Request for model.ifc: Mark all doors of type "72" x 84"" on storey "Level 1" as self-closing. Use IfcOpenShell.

First a look at what the model holds.

```python
import ifcopenshell
import ifcopenshell.util.element

model = ifcopenshell.open("model.ifc")
print(model.schema)
storey = next(s for s in model.by_type("IfcBuildingStorey") if s.Name == "Level 1")
doors = [e for e in ifcopenshell.util.element.get_decomposition(storey) if e.is_a("IfcDoor")]
seen = {}
for e in doors:
    element_type = ifcopenshell.util.element.get_type(e)
    key = (element_type.Name if element_type != e and element_type else None, ifcopenshell.util.element.get_pset(e, "Pset_DoorCommon", "SelfClosing"))
    seen[key] = seen.get(key, 0) + 1
for (name, value), count in sorted(seen.items(), key=str):
    print(count, "x", name, "|", value)
```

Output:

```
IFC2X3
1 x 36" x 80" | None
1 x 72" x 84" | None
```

```python
import ifcopenshell
import ifcopenshell.api.pset
import ifcopenshell.util.element

model = ifcopenshell.open("model.ifc")

storey = next(s for s in model.by_type("IfcBuildingStorey") if s.Name == "Level 1")
doors = [e for e in ifcopenshell.util.element.get_decomposition(storey) if e.is_a("IfcDoor")]

count = 0
for e in doors:
    element_type = ifcopenshell.util.element.get_type(e)
    if element_type in (None, e) or element_type.Name != '72" x 84"':
        continue
    # add_pset returns the element's existing set when there is one.
    pset = ifcopenshell.api.pset.add_pset(model, product=e, name="Pset_DoorCommon")
    ifcopenshell.api.pset.edit_pset(model, pset=pset, properties={"SelfClosing": True})
    count += 1

print(count, "doors updated")

model.write("model-out.ifc")
```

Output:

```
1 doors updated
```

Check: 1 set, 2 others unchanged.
